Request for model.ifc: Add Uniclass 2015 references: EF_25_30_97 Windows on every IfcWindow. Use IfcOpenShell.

First a look at what the model holds.

```python
import ifcopenshell

model = ifcopenshell.open("model.ifc")
print(model.schema)
print("classifications:", [c.Name for c in model.by_type("IfcClassification")])
for ifc_class in ("IfcDoor", "IfcRoof", "IfcStair", "IfcWall", "IfcWindow"):
    print(ifc_class, len(model.by_type(ifc_class)))
```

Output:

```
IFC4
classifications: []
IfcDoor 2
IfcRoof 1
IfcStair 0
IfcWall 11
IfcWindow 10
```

```python
import ifcopenshell
import ifcopenshell.api.classification

model = ifcopenshell.open("model.ifc")

system = ifcopenshell.api.classification.add_classification(model, classification="Uniclass 2015")

codes = {
    "IfcWindow": ("EF_25_30_97", "Windows"),
}
for ifc_class, (code, name) in codes.items():
    products = model.by_type(ifc_class)
    ifcopenshell.api.classification.add_reference(
        model, products=products, classification=system, identification=code, name=name
    )
    print(code, len(products))

model.write("model_edited.ifc")
```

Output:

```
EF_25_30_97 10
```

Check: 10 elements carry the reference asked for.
